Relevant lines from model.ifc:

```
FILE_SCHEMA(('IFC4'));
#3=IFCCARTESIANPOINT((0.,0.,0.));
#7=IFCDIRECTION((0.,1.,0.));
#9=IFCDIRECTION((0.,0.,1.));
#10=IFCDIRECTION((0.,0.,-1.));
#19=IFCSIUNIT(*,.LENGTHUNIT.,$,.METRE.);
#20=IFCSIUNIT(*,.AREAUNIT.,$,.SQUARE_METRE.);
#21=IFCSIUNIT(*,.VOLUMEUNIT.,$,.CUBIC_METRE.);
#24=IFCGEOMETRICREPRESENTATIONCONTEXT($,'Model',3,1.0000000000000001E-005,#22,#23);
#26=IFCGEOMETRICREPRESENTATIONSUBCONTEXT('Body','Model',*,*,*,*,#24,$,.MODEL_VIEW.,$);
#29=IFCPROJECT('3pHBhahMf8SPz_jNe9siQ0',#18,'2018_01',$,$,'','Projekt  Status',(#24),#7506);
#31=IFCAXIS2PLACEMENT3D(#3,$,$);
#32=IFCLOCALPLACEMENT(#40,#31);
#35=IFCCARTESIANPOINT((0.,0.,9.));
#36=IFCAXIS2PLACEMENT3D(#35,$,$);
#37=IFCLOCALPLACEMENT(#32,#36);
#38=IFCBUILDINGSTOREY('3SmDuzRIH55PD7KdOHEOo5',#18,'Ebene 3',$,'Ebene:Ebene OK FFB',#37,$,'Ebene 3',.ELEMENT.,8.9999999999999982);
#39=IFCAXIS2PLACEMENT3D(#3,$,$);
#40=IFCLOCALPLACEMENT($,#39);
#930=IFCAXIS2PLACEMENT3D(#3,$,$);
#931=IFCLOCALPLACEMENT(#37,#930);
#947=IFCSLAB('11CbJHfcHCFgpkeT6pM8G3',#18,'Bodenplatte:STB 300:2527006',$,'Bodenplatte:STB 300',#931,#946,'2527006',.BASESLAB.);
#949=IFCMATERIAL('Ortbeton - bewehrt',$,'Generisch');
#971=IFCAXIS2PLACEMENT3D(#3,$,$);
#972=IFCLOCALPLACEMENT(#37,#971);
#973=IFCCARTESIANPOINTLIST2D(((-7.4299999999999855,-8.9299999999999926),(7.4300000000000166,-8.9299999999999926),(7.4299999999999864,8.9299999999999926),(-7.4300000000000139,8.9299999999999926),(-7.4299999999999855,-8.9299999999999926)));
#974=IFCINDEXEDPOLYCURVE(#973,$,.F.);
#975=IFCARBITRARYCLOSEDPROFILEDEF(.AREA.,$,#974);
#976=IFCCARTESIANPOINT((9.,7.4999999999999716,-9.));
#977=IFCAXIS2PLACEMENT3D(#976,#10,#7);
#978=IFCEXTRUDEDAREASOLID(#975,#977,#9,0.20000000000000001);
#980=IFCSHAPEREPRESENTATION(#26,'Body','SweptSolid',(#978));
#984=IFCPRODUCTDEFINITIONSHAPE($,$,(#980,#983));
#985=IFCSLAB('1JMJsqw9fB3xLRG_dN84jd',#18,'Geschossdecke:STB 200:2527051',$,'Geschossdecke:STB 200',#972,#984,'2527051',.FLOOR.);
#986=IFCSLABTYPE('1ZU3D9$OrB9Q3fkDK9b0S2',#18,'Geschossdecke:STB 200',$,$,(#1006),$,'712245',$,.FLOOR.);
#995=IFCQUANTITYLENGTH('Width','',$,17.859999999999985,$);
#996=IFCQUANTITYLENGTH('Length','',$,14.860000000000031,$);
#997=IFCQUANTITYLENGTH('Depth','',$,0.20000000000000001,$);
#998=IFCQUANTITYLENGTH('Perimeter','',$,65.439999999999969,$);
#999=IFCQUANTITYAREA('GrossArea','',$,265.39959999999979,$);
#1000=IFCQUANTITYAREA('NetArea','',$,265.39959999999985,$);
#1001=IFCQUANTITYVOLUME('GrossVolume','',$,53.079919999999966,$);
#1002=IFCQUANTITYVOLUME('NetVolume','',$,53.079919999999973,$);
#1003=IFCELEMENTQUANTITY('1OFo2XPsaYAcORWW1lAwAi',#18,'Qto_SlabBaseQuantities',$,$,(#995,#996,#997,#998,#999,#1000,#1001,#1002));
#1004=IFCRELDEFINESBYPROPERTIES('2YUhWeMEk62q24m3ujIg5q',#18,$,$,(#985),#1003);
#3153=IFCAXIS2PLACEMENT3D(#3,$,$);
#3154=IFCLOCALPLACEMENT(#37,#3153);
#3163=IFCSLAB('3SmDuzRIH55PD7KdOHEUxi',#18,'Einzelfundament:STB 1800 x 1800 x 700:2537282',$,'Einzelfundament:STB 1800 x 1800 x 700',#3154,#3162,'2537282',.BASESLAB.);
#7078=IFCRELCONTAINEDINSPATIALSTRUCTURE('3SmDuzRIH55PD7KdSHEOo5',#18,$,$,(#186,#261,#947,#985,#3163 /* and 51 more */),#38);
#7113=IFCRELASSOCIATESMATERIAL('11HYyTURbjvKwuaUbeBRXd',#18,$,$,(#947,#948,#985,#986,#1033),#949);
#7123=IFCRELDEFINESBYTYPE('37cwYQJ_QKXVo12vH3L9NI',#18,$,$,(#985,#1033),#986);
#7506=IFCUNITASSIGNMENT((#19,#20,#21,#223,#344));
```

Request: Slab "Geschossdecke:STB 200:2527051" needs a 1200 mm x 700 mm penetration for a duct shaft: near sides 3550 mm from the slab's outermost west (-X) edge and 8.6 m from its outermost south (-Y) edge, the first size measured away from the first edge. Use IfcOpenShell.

```python
import numpy as np
import ifcopenshell
import ifcopenshell.api.feature
import ifcopenshell.api.geometry
import ifcopenshell.api.pset
import ifcopenshell.api.root
import ifcopenshell.geom
import ifcopenshell.util.element
import ifcopenshell.util.placement
import ifcopenshell.util.representation
import ifcopenshell.util.shape
import ifcopenshell.util.unit

model = ifcopenshell.open("model.ifc")
unit_scale = ifcopenshell.util.unit.calculate_unit_scale(model)
area_scale = ifcopenshell.util.unit.calculate_unit_scale(model, "AREAUNIT")
volume_scale = ifcopenshell.util.unit.calculate_unit_scale(model, "VOLUMEUNIT")
settings = ifcopenshell.geom.settings()


def volume(element):
    """Net volume in cubic metres, openings subtracted."""
    shape = ifcopenshell.geom.create_shape(settings, element)
    return ifcopenshell.util.shape.get_volume(shape.geometry)


slab = model.by_guid("1JMJsqw9fB3xLRG_dN84jd")
before = volume(slab)

# Extent in the slab's own axes, in metres. The edges named are its -X and -Y sides.
slab_shape = ifcopenshell.geom.create_shape(settings, slab)
vertices = ifcopenshell.util.shape.get_vertices(slab_shape.geometry)
x_min, y_min, bottom = vertices.min(axis=0)
top = vertices[:, 2].max()

opening = ifcopenshell.api.root.create_entity(model, ifc_class="IfcOpeningElement", name="Duct shaft opening", predefined_type="OPENING")
context = ifcopenshell.util.representation.get_context(model, "Model", "Body", "MODEL_VIEW")
width, depth = 1.2, 0.7
outline = [(0.0, 0.0), (width, 0.0), (width, depth), (0.0, depth), (0.0, 0.0)]
# Overshoot both faces by 50 mm so the cut is clean.
shape = ifcopenshell.api.geometry.add_slab_representation(
    model, context=context, depth=top - bottom + 0.1, polyline=outline
)
ifcopenshell.api.geometry.assign_representation(model, product=opening, representation=shape)

matrix = ifcopenshell.util.placement.get_local_placement(slab.ObjectPlacement)
matrix[:, 3] = matrix @ np.append(np.array([x_min + 3.55, y_min + 8.6, bottom - 0.05]) / unit_scale, 1.0)
ifcopenshell.api.geometry.edit_object_placement(model, product=opening, matrix=matrix, is_si=False)
ifcopenshell.api.feature.add_feature(model, feature=opening, element=slab)

after = volume(slab)

# Update the slab's stored quantities.
qto = model.by_id(ifcopenshell.util.element.get_pset(slab, "Qto_SlabBaseQuantities", should_inherit=False)["id"])
ifcopenshell.api.pset.edit_qto(model, qto=qto, properties={
    "NetArea": after / (top - bottom) / area_scale,
    "NetVolume": after / volume_scale,
})

print(f"slab volume {before:.3f} -> {after:.3f} m3")

model.write("model_edited.ifc")
```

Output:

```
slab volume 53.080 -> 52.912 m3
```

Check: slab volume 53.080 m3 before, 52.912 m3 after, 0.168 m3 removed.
